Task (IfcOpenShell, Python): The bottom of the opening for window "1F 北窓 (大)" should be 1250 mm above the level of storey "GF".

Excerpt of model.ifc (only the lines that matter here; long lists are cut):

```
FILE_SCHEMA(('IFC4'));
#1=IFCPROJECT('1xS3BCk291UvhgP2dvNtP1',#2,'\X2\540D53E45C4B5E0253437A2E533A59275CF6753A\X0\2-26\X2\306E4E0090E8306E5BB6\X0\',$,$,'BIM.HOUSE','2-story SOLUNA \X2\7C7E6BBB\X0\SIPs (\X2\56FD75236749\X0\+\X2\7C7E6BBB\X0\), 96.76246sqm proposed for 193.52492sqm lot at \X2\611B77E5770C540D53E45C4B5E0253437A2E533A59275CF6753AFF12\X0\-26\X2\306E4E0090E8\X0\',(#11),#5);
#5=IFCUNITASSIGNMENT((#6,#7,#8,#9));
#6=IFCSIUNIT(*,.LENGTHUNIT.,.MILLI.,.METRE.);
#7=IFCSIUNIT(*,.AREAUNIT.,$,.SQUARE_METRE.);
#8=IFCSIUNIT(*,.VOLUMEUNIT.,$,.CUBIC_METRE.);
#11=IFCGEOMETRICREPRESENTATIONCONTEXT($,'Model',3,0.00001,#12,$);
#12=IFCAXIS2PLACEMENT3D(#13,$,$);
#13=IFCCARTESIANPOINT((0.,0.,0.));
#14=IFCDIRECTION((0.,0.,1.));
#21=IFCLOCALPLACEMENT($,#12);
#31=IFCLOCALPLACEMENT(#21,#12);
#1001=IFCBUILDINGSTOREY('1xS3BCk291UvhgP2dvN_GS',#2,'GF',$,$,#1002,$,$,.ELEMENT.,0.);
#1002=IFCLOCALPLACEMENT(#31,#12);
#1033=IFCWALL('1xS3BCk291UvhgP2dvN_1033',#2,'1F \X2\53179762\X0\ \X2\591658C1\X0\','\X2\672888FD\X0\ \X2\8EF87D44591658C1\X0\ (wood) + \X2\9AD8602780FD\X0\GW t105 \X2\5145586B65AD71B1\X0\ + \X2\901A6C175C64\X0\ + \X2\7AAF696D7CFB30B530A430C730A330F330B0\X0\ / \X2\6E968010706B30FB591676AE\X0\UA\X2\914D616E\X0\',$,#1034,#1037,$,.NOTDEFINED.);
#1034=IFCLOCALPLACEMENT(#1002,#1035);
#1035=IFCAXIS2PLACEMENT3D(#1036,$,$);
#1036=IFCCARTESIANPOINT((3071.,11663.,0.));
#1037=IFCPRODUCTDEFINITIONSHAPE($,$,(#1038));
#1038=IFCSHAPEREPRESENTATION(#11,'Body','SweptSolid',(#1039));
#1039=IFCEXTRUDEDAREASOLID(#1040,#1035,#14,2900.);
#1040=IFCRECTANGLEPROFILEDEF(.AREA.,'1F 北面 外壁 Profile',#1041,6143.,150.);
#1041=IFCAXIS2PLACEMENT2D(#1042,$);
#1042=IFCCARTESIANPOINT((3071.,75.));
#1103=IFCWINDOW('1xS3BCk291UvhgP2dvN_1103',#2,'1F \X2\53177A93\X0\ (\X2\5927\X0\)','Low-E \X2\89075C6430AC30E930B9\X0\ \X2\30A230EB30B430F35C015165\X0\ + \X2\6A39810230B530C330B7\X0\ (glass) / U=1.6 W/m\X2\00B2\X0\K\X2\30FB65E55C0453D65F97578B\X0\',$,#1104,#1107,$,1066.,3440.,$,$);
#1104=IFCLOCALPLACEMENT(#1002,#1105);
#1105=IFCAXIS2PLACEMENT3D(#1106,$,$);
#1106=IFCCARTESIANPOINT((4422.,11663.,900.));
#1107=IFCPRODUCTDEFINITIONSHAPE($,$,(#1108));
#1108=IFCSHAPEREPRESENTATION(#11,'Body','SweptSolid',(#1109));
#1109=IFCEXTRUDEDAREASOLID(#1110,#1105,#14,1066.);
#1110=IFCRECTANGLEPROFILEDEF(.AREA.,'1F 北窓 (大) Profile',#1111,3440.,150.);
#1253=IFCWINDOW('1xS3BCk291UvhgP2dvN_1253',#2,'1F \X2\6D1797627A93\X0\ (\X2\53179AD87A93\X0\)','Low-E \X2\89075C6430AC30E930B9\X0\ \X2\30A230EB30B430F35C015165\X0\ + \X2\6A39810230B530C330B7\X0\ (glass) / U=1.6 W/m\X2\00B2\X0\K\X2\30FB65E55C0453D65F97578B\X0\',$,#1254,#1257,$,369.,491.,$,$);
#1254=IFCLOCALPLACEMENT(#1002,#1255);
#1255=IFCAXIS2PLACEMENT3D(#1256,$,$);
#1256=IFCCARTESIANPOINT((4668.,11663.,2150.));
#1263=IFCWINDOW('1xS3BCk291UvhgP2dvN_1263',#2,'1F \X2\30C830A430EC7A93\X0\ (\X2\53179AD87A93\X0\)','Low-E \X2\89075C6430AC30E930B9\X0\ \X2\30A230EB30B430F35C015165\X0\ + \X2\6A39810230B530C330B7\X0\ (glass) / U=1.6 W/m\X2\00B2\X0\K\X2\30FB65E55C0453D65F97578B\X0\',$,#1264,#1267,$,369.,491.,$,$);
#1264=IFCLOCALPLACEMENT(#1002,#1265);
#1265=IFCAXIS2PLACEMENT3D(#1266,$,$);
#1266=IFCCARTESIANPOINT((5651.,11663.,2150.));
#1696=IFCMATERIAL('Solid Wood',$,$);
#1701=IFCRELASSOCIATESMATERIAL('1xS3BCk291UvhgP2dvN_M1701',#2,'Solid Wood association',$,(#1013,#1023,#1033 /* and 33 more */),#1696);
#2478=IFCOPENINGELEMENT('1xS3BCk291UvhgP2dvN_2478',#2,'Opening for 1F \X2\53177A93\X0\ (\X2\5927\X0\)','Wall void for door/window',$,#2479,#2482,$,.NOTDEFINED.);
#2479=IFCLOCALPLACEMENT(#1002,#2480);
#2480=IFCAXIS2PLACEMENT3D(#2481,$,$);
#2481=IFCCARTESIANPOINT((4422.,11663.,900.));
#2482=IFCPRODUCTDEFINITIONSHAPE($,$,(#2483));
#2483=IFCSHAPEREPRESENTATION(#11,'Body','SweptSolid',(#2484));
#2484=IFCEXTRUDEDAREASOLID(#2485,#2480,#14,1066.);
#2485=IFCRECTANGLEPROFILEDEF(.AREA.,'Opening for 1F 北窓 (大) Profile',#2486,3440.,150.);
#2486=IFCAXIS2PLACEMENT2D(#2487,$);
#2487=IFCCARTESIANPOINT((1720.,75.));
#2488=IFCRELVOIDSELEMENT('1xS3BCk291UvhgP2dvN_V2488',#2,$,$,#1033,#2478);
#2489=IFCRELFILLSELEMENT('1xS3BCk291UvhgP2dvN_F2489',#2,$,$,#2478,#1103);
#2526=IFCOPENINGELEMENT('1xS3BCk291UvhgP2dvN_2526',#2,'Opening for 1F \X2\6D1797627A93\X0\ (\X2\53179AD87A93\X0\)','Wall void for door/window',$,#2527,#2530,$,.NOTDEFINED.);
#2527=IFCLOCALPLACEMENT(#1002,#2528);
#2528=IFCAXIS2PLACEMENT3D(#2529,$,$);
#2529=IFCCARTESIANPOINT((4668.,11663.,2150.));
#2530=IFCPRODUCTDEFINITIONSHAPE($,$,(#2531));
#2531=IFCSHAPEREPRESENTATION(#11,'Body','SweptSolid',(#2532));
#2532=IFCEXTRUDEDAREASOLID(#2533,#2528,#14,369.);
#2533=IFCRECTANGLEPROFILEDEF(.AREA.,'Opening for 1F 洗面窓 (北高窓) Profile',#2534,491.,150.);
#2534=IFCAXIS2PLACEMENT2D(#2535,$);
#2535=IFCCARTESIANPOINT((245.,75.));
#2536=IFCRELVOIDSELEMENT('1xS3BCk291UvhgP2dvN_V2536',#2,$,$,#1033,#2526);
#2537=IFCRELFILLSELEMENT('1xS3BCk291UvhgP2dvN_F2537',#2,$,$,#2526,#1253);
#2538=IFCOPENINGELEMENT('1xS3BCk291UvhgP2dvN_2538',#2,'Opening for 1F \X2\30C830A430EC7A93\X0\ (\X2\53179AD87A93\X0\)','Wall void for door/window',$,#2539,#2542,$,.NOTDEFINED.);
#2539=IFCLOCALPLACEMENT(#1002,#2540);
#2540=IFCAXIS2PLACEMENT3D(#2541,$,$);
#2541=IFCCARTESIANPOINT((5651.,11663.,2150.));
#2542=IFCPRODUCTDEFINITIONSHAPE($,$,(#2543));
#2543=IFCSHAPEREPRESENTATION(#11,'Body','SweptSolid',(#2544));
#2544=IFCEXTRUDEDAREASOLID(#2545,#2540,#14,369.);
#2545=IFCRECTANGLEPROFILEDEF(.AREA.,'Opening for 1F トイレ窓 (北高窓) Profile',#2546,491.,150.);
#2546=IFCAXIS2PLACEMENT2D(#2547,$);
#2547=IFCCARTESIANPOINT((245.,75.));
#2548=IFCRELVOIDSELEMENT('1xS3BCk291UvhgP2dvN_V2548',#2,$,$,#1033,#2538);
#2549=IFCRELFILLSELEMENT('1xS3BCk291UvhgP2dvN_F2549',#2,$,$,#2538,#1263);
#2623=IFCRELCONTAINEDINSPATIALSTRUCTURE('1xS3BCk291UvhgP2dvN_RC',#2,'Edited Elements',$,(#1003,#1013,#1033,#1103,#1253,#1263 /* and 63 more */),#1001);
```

```python
import numpy as np
import ifcopenshell
import ifcopenshell.api.geometry
import ifcopenshell.geom
import ifcopenshell.util.element
import ifcopenshell.util.placement
import ifcopenshell.util.shape
import ifcopenshell.util.unit

model = ifcopenshell.open("model.ifc")
unit_scale = ifcopenshell.util.unit.calculate_unit_scale(model)

window = model.by_id(1103)
opening = window.FillsVoids[0].RelatingOpeningElement
storey = ifcopenshell.util.element.get_container(window, ifc_class="IfcBuildingStorey")
level = ifcopenshell.util.placement.get_local_placement(storey.ObjectPlacement)[2, 3]

# The opening's origin need not be at the sill, so measure its lowest point.
shape = ifcopenshell.geom.create_shape(ifcopenshell.geom.settings(), opening)
bottom = ifcopenshell.util.shape.get_shape_bottom_elevation(shape, shape.geometry) / unit_scale
dz = level + 1250.0 - bottom

shift = np.array([0.0, 0.0, dz])
# The window is not placed relative to its opening, so move both.
for product in (opening, window):
    matrix = ifcopenshell.util.placement.get_local_placement(product.ObjectPlacement)
    matrix[:3, 3] += shift
    ifcopenshell.api.geometry.edit_object_placement(model, product=product, matrix=matrix, is_si=False)

print(f"moved by {dz * unit_scale:+.3f} m")

model.write("model_rev.ifc")
```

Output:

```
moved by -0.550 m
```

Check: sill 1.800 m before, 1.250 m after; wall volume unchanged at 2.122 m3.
